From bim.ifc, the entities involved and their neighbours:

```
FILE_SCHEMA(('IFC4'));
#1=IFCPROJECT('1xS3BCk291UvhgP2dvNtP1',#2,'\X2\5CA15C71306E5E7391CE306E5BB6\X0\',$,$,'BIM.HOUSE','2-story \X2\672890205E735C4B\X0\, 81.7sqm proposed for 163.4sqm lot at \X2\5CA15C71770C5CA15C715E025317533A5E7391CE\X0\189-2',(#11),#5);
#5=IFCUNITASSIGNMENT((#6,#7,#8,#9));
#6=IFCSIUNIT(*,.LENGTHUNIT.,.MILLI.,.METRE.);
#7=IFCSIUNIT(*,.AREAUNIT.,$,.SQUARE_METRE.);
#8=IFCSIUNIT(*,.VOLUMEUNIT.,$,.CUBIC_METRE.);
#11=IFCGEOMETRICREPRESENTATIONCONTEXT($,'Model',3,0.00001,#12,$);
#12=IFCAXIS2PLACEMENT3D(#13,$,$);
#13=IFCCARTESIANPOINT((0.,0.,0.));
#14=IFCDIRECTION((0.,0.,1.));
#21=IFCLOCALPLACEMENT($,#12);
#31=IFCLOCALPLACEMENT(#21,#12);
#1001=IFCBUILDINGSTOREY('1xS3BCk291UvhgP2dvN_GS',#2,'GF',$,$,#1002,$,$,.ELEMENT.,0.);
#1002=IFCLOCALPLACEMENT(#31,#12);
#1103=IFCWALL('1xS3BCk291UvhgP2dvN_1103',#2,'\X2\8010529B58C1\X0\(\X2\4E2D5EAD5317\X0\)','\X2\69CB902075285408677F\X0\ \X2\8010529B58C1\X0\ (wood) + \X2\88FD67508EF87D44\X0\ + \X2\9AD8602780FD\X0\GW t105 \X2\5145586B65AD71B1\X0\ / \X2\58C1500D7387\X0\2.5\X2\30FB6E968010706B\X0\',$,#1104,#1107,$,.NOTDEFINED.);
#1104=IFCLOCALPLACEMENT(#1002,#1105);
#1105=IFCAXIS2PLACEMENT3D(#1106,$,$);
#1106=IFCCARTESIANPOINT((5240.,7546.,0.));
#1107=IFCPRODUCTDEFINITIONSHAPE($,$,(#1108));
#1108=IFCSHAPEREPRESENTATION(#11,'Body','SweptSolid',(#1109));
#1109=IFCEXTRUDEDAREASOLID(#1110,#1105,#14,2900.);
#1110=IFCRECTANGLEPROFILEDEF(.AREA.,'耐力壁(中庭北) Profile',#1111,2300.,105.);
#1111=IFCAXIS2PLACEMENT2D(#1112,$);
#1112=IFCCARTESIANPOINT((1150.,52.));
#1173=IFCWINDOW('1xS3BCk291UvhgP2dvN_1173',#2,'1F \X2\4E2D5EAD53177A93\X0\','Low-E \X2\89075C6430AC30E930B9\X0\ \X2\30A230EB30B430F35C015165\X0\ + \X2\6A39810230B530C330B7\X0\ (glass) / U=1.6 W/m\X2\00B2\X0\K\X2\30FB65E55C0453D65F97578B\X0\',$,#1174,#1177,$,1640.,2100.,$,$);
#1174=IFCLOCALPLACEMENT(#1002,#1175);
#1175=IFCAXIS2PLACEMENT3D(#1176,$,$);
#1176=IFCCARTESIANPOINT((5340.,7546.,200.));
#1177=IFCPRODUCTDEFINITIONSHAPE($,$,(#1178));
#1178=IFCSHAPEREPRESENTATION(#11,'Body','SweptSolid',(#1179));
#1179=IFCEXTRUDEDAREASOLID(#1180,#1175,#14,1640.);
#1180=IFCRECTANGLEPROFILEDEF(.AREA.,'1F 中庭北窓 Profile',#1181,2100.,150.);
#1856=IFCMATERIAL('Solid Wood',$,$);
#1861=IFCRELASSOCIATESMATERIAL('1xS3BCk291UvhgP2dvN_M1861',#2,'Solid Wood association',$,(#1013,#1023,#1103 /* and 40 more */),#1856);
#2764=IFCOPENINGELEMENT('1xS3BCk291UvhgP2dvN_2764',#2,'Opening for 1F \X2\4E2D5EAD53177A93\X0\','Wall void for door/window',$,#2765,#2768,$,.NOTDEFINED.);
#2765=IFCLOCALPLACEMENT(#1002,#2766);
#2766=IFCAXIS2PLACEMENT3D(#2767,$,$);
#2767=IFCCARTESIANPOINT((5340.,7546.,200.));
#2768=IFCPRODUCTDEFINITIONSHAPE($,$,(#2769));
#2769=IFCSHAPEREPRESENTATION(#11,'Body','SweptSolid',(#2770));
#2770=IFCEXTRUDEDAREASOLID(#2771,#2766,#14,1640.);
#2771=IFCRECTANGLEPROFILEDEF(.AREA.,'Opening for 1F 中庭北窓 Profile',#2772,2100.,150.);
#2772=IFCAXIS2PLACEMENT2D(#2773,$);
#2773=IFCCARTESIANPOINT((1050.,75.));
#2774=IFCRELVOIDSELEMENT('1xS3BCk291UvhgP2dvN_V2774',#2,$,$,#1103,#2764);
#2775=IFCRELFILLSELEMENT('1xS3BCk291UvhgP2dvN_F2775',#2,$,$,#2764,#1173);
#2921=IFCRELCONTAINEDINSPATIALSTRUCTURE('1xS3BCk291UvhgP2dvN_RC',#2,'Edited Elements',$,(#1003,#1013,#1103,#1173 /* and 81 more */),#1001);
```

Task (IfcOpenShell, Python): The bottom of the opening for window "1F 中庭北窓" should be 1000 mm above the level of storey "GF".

```python
import numpy as np
import ifcopenshell
import ifcopenshell.api.geometry
import ifcopenshell.geom
import ifcopenshell.util.element
import ifcopenshell.util.placement
import ifcopenshell.util.shape
import ifcopenshell.util.unit

model = ifcopenshell.open("bim.ifc")
unit_scale = ifcopenshell.util.unit.calculate_unit_scale(model)

window = model.by_guid("1xS3BCk291UvhgP2dvN_1173")
opening = window.FillsVoids[0].RelatingOpeningElement
storey = ifcopenshell.util.element.get_container(window, ifc_class="IfcBuildingStorey")
level = ifcopenshell.util.placement.get_local_placement(storey.ObjectPlacement)[2, 3]

# The opening's origin need not be at the sill, so measure its lowest point.
shape = ifcopenshell.geom.create_shape(ifcopenshell.geom.settings(), opening)
bottom = ifcopenshell.util.shape.get_shape_bottom_elevation(shape, shape.geometry) / unit_scale
dz = level + 1000.0 - bottom

shift = np.array([0.0, 0.0, dz])
# The window is not placed relative to its opening, so move both.
for product in (opening, window):
    matrix = ifcopenshell.util.placement.get_local_placement(product.ObjectPlacement)
    matrix[:3, 3] += shift
    ifcopenshell.api.geometry.edit_object_placement(model, product=product, matrix=matrix, is_si=False)

print(f"moved by {dz * unit_scale:+.3f} m")

model.write("bim-out.ifc")
```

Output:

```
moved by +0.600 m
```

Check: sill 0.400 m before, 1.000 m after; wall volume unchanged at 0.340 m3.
